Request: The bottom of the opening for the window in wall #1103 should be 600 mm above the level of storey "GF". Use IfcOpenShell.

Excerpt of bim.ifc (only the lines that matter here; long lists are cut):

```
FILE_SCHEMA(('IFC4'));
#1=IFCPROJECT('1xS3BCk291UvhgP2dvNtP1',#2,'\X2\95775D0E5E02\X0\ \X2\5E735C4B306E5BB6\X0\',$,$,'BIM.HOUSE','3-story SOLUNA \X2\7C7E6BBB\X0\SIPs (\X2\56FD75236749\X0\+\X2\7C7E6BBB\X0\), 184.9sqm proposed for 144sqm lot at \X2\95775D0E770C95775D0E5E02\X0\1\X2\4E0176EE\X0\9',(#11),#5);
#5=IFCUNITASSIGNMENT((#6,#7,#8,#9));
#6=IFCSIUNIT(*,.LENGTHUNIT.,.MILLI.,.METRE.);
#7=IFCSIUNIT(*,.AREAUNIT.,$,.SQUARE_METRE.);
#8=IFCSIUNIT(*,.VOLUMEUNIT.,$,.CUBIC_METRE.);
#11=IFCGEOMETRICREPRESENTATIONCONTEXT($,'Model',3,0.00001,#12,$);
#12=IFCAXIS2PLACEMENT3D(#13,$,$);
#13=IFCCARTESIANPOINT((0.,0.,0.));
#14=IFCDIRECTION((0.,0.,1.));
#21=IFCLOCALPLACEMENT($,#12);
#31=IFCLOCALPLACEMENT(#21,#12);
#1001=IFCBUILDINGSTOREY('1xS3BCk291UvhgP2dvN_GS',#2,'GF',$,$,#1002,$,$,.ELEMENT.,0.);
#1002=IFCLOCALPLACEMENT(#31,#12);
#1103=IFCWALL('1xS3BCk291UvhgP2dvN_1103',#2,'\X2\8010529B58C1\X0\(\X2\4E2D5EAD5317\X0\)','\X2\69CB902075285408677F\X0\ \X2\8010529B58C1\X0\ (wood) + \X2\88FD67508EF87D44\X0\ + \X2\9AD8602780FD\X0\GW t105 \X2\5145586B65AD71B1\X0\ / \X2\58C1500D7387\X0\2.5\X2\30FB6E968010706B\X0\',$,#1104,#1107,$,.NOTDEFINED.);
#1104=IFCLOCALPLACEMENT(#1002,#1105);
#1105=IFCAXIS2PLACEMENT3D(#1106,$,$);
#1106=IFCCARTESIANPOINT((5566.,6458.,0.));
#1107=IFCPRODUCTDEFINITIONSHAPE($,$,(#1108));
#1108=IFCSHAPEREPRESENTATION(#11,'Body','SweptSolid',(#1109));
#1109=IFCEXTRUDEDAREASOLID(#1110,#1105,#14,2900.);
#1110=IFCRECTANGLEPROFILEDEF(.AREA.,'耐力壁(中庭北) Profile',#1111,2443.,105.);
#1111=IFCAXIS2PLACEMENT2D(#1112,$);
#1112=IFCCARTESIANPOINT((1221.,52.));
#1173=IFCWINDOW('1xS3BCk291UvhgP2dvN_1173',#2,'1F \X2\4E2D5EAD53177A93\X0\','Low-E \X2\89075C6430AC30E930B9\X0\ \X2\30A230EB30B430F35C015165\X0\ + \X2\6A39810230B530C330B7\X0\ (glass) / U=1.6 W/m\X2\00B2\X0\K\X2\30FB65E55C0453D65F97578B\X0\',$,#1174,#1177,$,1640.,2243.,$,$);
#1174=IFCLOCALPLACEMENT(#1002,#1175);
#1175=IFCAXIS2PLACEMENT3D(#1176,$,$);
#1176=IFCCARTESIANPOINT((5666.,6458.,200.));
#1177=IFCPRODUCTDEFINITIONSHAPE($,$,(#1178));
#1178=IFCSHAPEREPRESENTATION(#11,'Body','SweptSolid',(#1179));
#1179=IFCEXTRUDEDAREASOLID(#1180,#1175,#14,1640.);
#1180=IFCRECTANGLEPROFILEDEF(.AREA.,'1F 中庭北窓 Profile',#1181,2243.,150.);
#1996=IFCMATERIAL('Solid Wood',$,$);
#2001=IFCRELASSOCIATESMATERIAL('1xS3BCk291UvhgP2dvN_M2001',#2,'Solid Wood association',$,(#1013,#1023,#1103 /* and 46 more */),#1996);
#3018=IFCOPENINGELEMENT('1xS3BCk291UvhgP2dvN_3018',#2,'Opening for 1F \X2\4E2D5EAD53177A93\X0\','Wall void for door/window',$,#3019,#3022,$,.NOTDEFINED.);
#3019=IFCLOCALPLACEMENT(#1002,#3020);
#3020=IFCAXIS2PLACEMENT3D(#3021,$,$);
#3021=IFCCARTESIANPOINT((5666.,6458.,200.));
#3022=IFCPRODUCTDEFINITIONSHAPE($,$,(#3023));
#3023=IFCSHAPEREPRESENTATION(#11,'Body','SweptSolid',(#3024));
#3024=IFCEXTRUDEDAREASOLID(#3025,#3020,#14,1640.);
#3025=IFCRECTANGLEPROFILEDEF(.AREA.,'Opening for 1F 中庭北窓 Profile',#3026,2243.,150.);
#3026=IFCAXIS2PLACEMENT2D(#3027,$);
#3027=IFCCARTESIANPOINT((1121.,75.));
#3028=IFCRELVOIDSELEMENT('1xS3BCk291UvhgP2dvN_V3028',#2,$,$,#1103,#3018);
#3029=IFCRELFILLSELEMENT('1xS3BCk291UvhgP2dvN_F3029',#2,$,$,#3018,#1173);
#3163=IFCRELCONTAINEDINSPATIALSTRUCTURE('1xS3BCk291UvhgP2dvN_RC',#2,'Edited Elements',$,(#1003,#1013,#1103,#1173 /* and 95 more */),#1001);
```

```python
import numpy as np
import ifcopenshell
import ifcopenshell.api.geometry
import ifcopenshell.geom
import ifcopenshell.util.element
import ifcopenshell.util.placement
import ifcopenshell.util.shape
import ifcopenshell.util.unit

model = ifcopenshell.open("bim.ifc")
unit_scale = ifcopenshell.util.unit.calculate_unit_scale(model)

window = model.by_guid("1xS3BCk291UvhgP2dvN_1173")
opening = window.FillsVoids[0].RelatingOpeningElement
storey = ifcopenshell.util.element.get_container(window, ifc_class="IfcBuildingStorey")
level = ifcopenshell.util.placement.get_local_placement(storey.ObjectPlacement)[2, 3]

# The opening's origin need not be at the sill, so measure its lowest point.
shape = ifcopenshell.geom.create_shape(ifcopenshell.geom.settings(), opening)
bottom = ifcopenshell.util.shape.get_shape_bottom_elevation(shape, shape.geometry) / unit_scale
dz = level + 0.6 / unit_scale - bottom

shift = np.array([0.0, 0.0, dz])
# The window is not placed relative to its opening, so move both.
for product in (opening, window):
    matrix = ifcopenshell.util.placement.get_local_placement(product.ObjectPlacement)
    matrix[:3, 3] += shift
    ifcopenshell.api.geometry.edit_object_placement(model, product=product, matrix=matrix, is_si=False)

print(f"moved by {dz * unit_scale:+.3f} m")

model.write("bim_rev.ifc")
```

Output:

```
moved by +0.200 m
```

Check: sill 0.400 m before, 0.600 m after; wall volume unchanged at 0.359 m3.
